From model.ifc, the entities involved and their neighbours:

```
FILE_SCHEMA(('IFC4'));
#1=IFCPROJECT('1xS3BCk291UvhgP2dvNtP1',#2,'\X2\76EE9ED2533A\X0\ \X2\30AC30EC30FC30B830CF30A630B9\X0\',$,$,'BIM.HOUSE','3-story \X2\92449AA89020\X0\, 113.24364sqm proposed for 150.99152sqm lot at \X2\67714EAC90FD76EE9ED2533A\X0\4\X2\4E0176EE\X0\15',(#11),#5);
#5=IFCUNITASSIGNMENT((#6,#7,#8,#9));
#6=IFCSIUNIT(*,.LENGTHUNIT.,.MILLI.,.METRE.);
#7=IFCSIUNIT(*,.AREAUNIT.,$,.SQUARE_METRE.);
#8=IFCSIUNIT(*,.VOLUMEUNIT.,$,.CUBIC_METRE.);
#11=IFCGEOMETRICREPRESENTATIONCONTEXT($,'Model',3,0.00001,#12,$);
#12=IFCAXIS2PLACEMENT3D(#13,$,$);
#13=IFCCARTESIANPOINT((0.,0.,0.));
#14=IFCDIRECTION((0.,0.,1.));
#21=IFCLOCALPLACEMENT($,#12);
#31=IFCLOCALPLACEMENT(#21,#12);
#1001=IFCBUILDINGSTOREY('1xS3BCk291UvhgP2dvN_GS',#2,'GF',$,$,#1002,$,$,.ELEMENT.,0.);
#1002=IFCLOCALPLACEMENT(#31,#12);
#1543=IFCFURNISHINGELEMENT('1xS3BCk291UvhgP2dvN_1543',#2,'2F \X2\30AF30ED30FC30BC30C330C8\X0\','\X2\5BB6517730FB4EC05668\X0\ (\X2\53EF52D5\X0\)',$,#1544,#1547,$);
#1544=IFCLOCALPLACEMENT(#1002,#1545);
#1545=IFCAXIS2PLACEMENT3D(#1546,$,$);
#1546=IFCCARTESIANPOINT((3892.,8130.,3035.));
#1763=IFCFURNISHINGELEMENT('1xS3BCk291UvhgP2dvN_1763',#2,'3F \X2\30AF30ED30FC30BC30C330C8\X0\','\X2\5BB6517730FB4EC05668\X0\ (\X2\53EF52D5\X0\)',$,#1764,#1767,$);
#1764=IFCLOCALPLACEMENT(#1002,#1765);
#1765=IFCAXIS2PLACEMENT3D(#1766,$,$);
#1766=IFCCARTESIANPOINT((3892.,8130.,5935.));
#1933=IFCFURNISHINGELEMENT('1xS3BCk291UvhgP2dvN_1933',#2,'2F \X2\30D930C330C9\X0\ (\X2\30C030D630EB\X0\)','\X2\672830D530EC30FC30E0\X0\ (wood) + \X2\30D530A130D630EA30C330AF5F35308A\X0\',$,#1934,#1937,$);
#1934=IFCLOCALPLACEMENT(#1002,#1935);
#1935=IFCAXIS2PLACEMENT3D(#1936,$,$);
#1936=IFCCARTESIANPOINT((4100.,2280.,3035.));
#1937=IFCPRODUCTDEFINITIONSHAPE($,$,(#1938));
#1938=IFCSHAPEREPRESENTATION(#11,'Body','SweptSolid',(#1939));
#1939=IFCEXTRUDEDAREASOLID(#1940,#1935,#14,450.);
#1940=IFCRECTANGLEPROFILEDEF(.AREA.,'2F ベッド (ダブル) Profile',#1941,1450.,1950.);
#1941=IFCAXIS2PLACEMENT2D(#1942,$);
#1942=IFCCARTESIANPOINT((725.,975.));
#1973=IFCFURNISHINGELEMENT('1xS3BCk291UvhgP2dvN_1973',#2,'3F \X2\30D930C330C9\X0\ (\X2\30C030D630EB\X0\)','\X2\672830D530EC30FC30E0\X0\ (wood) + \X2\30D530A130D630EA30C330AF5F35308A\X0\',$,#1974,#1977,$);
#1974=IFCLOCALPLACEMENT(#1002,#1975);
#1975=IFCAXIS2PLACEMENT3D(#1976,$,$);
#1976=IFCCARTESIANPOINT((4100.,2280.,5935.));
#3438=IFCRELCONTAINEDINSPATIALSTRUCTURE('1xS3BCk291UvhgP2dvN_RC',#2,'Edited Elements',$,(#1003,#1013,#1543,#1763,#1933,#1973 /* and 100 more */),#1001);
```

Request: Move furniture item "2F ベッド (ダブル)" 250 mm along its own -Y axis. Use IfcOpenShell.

```python
import ifcopenshell
import ifcopenshell.api.geometry
import ifcopenshell.util.placement
import ifcopenshell.util.unit

model = ifcopenshell.open("model.ifc")
unit_scale = ifcopenshell.util.unit.calculate_unit_scale(model)

item = model.by_guid("1xS3BCk291UvhgP2dvN_1933")
matrix = ifcopenshell.util.placement.get_local_placement(item.ObjectPlacement)
matrix[:3, 3] -= matrix[:3, 1] * 0.25 / unit_scale
ifcopenshell.api.geometry.edit_object_placement(model, product=item, matrix=matrix, is_si=False)

print(ifcopenshell.util.placement.get_local_placement(item.ObjectPlacement).round(3) + 0.0)

model.write("model_edited.ifc")
```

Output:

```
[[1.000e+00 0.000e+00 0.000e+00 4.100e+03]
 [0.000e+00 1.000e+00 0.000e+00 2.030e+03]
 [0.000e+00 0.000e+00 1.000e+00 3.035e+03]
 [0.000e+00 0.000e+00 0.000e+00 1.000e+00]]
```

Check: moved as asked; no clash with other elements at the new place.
